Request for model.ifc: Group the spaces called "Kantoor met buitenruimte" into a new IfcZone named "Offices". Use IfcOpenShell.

First a look at what the model holds.

```python
import ifcopenshell

model = ifcopenshell.open("model.ifc")
print(model.schema)
seen = {}
for space in model.by_type("IfcSpace"):
    seen[space.LongName] = seen.get(space.LongName, 0) + 1
for name, count in sorted(seen.items(), key=str):
    print(count, "x", name)
print("zones:", [z.Name for z in model.by_type("IfcZone")][:20])
```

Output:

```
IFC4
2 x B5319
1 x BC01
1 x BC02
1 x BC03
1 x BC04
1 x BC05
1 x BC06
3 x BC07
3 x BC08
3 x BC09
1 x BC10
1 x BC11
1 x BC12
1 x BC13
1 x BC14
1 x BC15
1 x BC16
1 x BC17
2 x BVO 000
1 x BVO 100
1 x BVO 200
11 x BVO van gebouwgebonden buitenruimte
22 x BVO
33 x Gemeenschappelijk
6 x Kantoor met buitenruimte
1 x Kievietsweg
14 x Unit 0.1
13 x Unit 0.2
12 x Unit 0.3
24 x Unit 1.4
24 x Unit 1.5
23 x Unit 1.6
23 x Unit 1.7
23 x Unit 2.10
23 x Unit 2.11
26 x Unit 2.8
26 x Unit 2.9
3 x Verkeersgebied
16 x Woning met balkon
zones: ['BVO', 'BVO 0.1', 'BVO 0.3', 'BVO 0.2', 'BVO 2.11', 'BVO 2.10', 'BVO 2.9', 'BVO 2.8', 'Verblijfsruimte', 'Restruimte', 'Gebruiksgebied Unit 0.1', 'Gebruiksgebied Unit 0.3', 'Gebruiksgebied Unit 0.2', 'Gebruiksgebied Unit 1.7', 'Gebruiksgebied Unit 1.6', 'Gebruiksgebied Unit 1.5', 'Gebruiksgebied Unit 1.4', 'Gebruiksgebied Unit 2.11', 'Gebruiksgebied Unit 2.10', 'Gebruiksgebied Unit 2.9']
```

```python
import ifcopenshell
import ifcopenshell.api.group
import ifcopenshell.api.root

model = ifcopenshell.open("model.ifc")

names = {"Kantoor met buitenruimte"}
spaces = [s for s in model.by_type("IfcSpace") if s.LongName in names]

zone = ifcopenshell.api.root.create_entity(model, ifc_class="IfcZone", name="Offices")
ifcopenshell.api.group.assign_group(model, products=spaces, group=zone)
print(len(spaces), "spaces in", zone.Name)

model.write("model_edited.ifc")
```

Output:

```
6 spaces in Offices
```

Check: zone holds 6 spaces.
